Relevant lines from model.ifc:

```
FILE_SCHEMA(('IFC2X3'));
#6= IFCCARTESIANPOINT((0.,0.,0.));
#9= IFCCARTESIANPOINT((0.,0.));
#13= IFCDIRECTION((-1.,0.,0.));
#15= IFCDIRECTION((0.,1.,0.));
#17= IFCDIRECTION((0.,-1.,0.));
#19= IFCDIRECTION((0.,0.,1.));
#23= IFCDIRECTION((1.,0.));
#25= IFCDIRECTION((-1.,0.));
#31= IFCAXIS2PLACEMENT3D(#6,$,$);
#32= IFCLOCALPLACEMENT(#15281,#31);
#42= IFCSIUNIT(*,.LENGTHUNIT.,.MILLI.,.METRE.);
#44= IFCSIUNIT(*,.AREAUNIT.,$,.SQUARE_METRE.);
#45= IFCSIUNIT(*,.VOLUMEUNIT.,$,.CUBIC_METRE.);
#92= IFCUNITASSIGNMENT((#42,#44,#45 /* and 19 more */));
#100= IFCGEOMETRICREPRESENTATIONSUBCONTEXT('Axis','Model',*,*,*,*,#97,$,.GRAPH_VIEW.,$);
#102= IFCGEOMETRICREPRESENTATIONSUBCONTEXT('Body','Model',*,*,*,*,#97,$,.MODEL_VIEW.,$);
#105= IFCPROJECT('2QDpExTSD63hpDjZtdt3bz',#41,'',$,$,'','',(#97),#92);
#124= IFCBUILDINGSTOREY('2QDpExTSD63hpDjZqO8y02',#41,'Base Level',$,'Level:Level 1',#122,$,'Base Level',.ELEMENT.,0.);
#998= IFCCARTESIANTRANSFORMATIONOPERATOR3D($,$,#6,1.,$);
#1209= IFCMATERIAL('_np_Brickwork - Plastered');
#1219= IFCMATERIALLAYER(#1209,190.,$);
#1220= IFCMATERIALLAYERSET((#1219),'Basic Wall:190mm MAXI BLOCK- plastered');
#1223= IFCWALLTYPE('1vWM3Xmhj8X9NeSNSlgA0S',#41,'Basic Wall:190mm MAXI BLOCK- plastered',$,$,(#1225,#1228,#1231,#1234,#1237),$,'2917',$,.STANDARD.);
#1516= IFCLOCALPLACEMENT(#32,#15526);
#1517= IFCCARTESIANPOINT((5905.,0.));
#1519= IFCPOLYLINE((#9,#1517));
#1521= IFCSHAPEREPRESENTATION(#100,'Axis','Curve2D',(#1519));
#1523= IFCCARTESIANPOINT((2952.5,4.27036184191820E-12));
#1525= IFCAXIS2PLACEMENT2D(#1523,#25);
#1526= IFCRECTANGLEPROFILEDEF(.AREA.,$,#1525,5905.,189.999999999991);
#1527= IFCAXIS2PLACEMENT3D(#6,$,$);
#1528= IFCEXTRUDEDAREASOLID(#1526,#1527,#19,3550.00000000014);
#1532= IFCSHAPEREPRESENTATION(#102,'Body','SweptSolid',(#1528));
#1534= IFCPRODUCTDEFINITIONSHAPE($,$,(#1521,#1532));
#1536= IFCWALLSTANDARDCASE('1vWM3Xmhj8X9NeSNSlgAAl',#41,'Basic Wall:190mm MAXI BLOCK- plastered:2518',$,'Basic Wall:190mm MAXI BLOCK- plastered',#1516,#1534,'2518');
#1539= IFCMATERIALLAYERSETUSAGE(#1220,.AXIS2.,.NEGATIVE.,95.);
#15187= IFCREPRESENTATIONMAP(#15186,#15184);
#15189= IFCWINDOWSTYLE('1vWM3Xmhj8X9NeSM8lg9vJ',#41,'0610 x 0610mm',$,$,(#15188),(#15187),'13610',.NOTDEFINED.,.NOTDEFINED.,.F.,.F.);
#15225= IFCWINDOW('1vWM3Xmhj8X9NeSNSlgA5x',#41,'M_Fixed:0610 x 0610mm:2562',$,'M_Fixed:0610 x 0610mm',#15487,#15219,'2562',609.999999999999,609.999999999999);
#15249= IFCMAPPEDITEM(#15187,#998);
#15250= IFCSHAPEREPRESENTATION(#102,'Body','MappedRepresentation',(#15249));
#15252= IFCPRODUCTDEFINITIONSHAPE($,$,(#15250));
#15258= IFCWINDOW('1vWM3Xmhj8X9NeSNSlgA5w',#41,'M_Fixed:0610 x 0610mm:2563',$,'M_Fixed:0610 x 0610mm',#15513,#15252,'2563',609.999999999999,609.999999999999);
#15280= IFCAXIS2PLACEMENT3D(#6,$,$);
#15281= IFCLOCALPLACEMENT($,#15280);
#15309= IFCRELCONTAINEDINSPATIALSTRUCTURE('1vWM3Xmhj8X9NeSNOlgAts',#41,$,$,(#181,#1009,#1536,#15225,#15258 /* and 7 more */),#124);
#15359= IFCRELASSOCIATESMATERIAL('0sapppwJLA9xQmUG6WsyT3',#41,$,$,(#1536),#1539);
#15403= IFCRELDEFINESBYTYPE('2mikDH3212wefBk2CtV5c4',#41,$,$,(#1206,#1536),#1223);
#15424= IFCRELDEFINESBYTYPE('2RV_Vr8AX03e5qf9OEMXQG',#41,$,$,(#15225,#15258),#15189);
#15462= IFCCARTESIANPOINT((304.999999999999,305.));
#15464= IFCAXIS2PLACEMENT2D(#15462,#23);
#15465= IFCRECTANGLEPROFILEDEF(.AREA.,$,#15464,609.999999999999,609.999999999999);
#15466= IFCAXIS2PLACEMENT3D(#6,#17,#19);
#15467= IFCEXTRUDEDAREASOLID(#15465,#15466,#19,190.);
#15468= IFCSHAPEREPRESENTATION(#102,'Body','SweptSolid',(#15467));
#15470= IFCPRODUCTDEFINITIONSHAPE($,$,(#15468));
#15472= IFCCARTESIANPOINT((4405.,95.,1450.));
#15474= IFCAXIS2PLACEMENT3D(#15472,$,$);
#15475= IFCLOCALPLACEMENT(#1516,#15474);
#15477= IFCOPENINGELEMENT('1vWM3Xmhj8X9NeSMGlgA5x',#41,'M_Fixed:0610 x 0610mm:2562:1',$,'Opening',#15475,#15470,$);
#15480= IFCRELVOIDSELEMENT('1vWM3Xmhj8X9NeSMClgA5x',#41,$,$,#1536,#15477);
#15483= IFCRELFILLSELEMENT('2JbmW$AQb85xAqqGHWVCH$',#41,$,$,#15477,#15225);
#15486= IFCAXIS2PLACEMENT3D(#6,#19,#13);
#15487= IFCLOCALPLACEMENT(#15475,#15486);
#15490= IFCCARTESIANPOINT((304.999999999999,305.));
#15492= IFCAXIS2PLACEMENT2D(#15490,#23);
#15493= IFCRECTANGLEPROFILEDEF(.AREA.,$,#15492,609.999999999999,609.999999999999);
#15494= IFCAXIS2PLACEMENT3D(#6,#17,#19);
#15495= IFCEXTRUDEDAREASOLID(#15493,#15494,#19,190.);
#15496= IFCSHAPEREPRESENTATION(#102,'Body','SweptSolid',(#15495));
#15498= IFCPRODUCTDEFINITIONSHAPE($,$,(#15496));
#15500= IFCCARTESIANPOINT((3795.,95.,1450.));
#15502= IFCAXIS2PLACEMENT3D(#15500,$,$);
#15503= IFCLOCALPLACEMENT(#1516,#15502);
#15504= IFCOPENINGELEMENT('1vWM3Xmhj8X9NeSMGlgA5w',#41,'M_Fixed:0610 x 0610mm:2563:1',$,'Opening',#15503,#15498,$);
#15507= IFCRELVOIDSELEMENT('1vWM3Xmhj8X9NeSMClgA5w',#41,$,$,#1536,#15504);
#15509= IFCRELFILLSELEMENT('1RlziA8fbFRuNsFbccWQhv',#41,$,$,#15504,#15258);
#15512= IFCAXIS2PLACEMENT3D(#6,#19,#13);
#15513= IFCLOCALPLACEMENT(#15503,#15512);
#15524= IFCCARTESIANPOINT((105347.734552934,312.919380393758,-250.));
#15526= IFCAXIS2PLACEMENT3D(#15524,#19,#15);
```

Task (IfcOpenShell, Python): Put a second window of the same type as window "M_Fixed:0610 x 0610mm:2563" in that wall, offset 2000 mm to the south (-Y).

```python
import ifcopenshell
import ifcopenshell.api.feature
import ifcopenshell.api.geometry
import ifcopenshell.api.root
import ifcopenshell.geom
import ifcopenshell.util.element
import ifcopenshell.util.placement
import ifcopenshell.util.shape
import ifcopenshell.util.unit

model = ifcopenshell.open("model.ifc")
unit_scale = ifcopenshell.util.unit.calculate_unit_scale(model)
settings = ifcopenshell.geom.settings()


def volume(element):
    """Net volume in cubic metres, openings subtracted."""
    shape = ifcopenshell.geom.create_shape(settings, element)
    return ifcopenshell.util.shape.get_volume(shape.geometry)


def reuse_history(source, copy):
    """copy_class also copies each property set's owner history, people and application; keep the originals."""
    for rel in copy.IsDefinedBy:
        if rel.is_a("IfcRelDefinesByProperties") and (history := rel.RelatingPropertyDefinition.OwnerHistory):
            rel.RelatingPropertyDefinition.OwnerHistory = source.OwnerHistory
            ifcopenshell.util.element.remove_deep2(model, history)


window = model.by_guid("1vWM3Xmhj8X9NeSNSlgA5w")
opening = window.FillsVoids[0].RelatingOpeningElement
wall = opening.VoidsElements[0].RelatingBuildingElement
before = volume(wall)
shift = ifcopenshell.util.placement.get_local_placement(wall.ObjectPlacement)[:3, 0] * -2 / unit_scale

# copy_class copies the void relationship, type, container and properties, but no geometry.
new_opening = ifcopenshell.api.root.copy_class(model, product=opening)
new_opening.Representation = ifcopenshell.util.element.copy_deep(
    model, opening.Representation, exclude=["IfcGeometricRepresentationContext", "IfcRepresentationMap"]
)
new_opening.Name = "M_Fixed:0610 x 0610mm"
new_window = ifcopenshell.api.root.copy_class(model, product=window)
new_window.Representation = ifcopenshell.util.element.copy_deep(
    model, window.Representation, exclude=["IfcGeometricRepresentationContext", "IfcRepresentationMap"]
)
new_window.Name = "M_Fixed:0610 x 0610mm"
new_window.Tag = None
reuse_history(window, new_window)
fills = ifcopenshell.api.feature.add_filling(model, opening=new_opening, element=new_window)
fills.OwnerHistory = new_window.OwnerHistory  # required in IFC2X3

for old, new in ((opening, new_opening), (window, new_window)):
    matrix = ifcopenshell.util.placement.get_local_placement(old.ObjectPlacement)
    matrix[:3, 3] += shift
    ifcopenshell.api.geometry.edit_object_placement(model, product=new, matrix=matrix, is_si=False)

after = volume(wall)

print(f"wall volume {before:.3f} -> {after:.3f} m3")

model.write("model_updated.ifc")
```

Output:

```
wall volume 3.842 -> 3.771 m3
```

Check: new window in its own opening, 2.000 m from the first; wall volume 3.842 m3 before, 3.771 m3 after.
